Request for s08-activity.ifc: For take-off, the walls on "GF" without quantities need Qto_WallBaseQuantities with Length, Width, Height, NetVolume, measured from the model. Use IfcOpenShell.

First a look at what the model holds.

```python
import ifcopenshell
import ifcopenshell.util.element
import ifcopenshell.util.unit

model = ifcopenshell.open("s08-activity.ifc")
print(model.schema)
for unit_type in ("LENGTHUNIT", "AREAUNIT", "VOLUMEUNIT"):
    print(unit_type, ifcopenshell.util.unit.calculate_unit_scale(model, unit_type))
storey = next(s for s in model.by_type("IfcBuildingStorey") if s.Name == "GF")
walls = [e for e in ifcopenshell.util.element.get_decomposition(storey) if e.is_a("IfcWall")]
for e in sorted(walls, key=lambda e: e.id()):
    print(e.id(), e.is_a(), e.Name, list(ifcopenshell.util.element.get_psets(e, qtos_only=True)), sep=" | ")
```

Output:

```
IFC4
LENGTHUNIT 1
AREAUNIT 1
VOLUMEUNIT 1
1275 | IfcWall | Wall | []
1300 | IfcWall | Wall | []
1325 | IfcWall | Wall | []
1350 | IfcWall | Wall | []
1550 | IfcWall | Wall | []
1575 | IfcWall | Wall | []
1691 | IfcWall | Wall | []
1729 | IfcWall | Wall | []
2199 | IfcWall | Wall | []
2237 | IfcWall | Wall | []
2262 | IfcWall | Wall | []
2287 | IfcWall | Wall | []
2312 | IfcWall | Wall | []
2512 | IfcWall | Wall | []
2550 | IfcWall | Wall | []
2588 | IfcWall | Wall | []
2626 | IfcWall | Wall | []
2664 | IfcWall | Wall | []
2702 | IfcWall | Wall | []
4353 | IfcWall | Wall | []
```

```python
import ifcopenshell
import ifcopenshell.api.pset
import ifcopenshell.geom
import ifcopenshell.util.element
import ifcopenshell.util.shape
import ifcopenshell.util.unit

model = ifcopenshell.open("s08-activity.ifc")
unit_scale = ifcopenshell.util.unit.calculate_unit_scale(model)
volume_scale = ifcopenshell.util.unit.calculate_unit_scale(model, "VOLUMEUNIT")
settings = ifcopenshell.geom.settings()

storey = next(s for s in model.by_type("IfcBuildingStorey") if s.Name == "GF")
walls = [e for e in ifcopenshell.util.element.get_decomposition(storey) if e.is_a("IfcWall")]

for e in sorted(walls, key=lambda e: e.id()):
    if ifcopenshell.util.element.get_psets(e, qtos_only=True, should_inherit=False):
        continue
    # Geometry comes back in metres, in the element's own axes.
    shape = ifcopenshell.geom.create_shape(settings, e)
    values = {
        "Length": ifcopenshell.util.shape.get_x(shape.geometry) / unit_scale,
        "Width": ifcopenshell.util.shape.get_y(shape.geometry) / unit_scale,
        "Height": ifcopenshell.util.shape.get_z(shape.geometry) / unit_scale,
        "NetVolume": ifcopenshell.util.shape.get_volume(shape.geometry) / volume_scale,
    }
    qto = ifcopenshell.api.pset.add_qto(model, product=e, name="Qto_WallBaseQuantities")
    ifcopenshell.api.pset.edit_qto(model, qto=qto, properties=values)
    print(e.id(), {k: round(v, 3) for k, v in values.items()})

model.write("s08-activity_v2.ifc")
```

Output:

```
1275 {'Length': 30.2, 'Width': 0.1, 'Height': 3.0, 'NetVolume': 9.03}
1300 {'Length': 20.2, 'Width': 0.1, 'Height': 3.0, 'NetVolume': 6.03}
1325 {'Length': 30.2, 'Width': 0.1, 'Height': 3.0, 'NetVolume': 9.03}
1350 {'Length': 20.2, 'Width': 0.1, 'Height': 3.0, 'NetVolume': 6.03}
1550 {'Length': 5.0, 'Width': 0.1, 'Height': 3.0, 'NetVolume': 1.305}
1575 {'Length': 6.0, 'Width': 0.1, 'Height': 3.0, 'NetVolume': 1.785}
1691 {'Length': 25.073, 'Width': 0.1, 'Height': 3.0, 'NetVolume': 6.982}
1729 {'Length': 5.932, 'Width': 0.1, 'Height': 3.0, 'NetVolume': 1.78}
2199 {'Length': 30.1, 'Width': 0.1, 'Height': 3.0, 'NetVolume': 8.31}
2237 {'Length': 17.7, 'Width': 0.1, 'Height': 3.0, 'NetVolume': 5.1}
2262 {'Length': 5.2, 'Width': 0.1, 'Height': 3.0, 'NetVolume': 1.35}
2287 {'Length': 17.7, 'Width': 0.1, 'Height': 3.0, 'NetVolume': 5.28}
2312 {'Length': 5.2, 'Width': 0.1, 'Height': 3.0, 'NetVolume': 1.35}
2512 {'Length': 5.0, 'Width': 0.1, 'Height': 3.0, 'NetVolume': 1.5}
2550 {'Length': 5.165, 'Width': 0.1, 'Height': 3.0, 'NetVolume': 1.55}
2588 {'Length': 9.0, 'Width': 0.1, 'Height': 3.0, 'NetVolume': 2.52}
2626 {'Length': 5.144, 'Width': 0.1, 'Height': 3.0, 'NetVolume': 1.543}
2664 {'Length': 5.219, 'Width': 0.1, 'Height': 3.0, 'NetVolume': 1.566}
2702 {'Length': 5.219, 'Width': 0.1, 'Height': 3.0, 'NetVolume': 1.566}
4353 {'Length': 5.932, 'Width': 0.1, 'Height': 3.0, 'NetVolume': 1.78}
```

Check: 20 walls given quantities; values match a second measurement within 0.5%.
